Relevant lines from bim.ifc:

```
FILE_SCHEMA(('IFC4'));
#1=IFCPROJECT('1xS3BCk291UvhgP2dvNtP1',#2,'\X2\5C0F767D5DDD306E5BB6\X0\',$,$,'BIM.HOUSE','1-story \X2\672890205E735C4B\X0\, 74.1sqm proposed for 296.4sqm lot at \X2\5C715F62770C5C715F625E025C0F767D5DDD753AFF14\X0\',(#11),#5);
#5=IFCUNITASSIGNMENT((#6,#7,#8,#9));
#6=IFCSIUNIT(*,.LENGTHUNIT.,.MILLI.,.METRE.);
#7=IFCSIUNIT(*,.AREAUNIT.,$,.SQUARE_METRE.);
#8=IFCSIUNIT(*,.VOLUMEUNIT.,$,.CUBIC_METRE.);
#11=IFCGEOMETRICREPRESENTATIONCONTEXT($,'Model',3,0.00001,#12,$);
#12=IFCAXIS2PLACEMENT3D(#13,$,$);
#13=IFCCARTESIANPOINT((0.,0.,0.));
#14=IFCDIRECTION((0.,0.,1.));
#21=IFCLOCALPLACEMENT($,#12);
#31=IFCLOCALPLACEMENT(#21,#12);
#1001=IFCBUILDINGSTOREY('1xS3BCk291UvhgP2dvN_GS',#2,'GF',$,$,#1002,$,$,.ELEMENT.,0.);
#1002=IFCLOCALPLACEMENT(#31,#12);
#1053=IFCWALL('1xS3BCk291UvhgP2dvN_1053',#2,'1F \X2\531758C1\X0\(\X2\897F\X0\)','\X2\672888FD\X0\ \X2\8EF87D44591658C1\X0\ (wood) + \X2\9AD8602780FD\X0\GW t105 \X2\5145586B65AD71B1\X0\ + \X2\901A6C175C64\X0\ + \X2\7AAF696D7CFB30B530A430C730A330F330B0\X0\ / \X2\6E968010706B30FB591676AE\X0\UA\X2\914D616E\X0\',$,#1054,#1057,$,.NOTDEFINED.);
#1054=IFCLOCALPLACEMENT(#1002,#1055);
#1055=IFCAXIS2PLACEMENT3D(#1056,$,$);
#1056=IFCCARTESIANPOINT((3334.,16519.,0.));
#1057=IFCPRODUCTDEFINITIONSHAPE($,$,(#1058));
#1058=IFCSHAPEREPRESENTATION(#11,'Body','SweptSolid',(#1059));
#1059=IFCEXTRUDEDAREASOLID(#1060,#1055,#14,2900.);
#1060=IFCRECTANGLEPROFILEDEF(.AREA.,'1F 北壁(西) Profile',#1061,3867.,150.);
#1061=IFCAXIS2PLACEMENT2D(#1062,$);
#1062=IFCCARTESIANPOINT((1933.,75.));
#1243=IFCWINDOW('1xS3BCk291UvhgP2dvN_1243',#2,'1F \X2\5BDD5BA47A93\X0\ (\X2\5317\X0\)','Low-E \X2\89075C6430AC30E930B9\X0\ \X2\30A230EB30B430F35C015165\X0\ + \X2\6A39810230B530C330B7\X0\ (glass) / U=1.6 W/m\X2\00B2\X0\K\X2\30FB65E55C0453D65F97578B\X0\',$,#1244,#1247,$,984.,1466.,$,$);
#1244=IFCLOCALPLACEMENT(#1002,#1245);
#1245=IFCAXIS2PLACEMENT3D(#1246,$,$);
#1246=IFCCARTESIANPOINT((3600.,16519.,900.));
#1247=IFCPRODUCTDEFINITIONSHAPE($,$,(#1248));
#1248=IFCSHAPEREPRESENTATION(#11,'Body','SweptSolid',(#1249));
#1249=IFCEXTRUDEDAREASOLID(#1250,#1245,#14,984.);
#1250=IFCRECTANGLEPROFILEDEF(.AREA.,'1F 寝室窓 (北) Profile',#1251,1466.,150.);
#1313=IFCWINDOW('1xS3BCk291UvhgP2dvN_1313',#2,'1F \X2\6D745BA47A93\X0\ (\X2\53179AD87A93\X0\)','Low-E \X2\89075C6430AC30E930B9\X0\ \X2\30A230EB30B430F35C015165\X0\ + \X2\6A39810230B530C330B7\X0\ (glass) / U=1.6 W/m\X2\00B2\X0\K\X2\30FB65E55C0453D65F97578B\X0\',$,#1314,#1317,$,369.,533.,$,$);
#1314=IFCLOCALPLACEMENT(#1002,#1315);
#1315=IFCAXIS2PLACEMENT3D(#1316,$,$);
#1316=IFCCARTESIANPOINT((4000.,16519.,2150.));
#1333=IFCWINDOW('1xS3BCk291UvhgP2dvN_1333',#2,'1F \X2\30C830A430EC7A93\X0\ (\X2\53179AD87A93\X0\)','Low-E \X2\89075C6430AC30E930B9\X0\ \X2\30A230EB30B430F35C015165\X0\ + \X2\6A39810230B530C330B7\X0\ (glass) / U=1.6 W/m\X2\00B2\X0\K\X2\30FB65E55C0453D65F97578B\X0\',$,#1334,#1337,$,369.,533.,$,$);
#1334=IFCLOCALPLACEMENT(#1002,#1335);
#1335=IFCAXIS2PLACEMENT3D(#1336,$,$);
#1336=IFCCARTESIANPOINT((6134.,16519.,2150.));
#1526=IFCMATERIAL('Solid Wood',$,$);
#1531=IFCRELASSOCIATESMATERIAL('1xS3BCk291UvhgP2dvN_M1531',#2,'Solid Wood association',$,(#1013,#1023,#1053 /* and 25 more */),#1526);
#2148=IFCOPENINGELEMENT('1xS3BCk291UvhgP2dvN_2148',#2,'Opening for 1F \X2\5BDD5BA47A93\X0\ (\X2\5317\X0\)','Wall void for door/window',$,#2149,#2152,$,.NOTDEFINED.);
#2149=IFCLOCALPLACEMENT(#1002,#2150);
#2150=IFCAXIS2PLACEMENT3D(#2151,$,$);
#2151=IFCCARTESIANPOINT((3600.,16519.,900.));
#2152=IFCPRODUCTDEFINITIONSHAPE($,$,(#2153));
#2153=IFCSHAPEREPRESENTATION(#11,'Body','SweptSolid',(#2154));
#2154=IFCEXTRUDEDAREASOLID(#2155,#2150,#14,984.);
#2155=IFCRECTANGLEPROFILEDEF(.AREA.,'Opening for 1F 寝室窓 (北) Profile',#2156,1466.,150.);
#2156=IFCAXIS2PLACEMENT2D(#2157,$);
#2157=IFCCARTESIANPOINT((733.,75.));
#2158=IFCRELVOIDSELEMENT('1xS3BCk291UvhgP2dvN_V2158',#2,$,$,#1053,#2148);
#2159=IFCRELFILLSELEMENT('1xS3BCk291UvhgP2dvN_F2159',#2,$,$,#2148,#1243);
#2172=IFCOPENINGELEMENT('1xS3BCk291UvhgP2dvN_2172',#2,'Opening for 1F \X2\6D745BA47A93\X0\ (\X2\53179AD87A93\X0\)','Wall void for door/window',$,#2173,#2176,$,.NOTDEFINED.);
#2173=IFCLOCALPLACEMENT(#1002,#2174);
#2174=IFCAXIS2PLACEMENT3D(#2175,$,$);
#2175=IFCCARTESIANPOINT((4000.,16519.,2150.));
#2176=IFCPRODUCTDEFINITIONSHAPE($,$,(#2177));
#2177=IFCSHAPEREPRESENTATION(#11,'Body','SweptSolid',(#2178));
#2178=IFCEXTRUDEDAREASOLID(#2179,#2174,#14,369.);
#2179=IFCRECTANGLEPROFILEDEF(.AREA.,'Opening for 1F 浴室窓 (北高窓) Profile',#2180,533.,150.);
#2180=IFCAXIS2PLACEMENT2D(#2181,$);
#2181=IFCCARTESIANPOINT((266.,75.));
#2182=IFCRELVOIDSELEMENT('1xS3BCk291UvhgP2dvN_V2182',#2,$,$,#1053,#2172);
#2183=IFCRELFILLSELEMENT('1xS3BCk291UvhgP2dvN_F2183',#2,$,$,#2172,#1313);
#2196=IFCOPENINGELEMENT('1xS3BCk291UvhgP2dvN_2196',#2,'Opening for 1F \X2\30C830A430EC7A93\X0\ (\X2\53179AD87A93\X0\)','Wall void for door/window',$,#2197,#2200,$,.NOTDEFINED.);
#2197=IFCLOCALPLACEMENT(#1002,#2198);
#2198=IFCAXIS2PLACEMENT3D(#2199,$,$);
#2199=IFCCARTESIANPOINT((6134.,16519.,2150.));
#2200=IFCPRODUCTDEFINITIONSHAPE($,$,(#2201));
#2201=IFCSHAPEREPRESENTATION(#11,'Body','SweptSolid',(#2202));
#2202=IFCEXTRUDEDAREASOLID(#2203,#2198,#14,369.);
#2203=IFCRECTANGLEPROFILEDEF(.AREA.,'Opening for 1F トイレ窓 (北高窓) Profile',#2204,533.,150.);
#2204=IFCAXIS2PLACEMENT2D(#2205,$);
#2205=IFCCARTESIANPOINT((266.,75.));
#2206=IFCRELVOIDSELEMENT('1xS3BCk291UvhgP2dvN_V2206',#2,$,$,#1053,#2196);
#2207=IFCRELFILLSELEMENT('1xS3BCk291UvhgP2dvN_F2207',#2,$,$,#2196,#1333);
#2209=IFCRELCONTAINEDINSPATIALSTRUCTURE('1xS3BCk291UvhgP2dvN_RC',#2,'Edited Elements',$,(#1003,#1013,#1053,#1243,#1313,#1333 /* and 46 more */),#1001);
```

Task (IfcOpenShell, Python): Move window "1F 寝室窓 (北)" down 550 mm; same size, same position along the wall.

```python
import numpy as np
import ifcopenshell
import ifcopenshell.api.geometry
import ifcopenshell.util.placement
import ifcopenshell.util.unit

model = ifcopenshell.open("bim.ifc")
unit_scale = ifcopenshell.util.unit.calculate_unit_scale(model)

window = model.by_guid("1xS3BCk291UvhgP2dvN_1243")
opening = window.FillsVoids[0].RelatingOpeningElement
dz = -550.0

shift = np.array([0.0, 0.0, dz])
# The window is not placed relative to its opening, so move both.
for product in (opening, window):
    matrix = ifcopenshell.util.placement.get_local_placement(product.ObjectPlacement)
    matrix[:3, 3] += shift
    ifcopenshell.api.geometry.edit_object_placement(model, product=product, matrix=matrix, is_si=False)

print(f"moved by {dz * unit_scale:+.3f} m")

model.write("bim_v2.ifc")
```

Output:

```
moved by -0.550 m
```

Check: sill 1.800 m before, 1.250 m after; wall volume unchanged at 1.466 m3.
